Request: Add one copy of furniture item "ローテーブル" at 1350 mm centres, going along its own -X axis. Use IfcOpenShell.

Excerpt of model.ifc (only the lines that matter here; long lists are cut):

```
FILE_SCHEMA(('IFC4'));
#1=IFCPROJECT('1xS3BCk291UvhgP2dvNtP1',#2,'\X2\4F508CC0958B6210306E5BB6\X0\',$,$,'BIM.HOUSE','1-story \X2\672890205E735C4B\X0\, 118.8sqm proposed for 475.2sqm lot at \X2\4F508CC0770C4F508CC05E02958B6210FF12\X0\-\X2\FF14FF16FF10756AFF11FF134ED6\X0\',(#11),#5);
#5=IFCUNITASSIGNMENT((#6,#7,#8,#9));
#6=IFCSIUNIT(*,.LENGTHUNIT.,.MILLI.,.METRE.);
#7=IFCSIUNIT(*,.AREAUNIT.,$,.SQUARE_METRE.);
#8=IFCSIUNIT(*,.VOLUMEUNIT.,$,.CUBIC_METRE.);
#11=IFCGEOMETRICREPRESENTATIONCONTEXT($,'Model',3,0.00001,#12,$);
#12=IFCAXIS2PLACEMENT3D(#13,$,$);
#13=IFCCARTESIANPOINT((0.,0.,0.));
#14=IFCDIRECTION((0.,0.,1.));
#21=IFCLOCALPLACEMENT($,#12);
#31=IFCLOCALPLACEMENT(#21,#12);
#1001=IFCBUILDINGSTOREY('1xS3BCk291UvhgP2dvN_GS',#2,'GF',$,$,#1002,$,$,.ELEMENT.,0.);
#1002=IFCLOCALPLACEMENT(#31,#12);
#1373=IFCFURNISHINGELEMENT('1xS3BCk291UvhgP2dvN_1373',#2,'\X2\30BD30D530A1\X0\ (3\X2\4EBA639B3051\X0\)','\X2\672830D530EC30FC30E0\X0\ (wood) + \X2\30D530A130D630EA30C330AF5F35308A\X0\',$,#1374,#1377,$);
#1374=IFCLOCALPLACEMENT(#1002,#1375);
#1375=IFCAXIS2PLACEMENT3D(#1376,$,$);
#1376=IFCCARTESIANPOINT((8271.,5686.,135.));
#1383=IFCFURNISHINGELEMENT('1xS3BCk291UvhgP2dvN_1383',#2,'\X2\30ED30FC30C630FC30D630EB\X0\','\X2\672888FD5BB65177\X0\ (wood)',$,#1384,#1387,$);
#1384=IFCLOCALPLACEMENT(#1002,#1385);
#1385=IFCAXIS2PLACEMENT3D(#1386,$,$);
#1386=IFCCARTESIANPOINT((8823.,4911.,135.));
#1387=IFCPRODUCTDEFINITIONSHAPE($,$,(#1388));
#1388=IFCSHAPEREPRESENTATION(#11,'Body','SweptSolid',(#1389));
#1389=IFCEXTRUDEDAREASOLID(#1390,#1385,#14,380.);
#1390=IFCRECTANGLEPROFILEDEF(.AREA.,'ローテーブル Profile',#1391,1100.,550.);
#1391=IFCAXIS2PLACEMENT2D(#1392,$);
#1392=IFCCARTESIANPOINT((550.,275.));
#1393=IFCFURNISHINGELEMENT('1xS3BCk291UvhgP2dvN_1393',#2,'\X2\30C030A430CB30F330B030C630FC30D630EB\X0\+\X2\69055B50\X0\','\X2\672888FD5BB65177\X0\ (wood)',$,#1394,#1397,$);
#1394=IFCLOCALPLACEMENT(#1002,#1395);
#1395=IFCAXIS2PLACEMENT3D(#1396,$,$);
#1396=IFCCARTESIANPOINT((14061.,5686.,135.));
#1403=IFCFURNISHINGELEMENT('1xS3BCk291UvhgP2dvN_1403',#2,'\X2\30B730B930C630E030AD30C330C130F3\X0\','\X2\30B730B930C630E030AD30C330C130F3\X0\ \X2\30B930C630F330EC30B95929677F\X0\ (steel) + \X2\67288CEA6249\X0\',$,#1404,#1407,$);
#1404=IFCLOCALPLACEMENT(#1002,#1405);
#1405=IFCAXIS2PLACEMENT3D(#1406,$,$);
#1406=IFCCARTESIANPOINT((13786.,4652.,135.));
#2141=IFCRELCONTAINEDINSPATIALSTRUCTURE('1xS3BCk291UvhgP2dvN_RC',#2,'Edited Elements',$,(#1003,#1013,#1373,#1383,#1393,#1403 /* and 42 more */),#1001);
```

```python
import ifcopenshell
import ifcopenshell.api.geometry
import ifcopenshell.api.root
import ifcopenshell.util.element
import ifcopenshell.util.placement
import ifcopenshell.util.unit

model = ifcopenshell.open("model.ifc")
unit_scale = ifcopenshell.util.unit.calculate_unit_scale(model)


def reuse_history(source, copy):
    """copy_class also copies each property set's owner history, people and application; keep the originals."""
    for rel in copy.IsDefinedBy:
        if rel.is_a("IfcRelDefinesByProperties") and (history := rel.RelatingPropertyDefinition.OwnerHistory):
            rel.RelatingPropertyDefinition.OwnerHistory = source.OwnerHistory
            ifcopenshell.util.element.remove_deep2(model, history)


source = model.by_guid("1xS3BCk291UvhgP2dvN_1383")
base = ifcopenshell.util.placement.get_local_placement(source.ObjectPlacement)
step = -base[:3, 0] * 1.35 / unit_scale

for i in range(1, 2):
    copy = ifcopenshell.api.root.copy_class(model, product=source)
    copy.Representation = ifcopenshell.util.element.copy_deep(
        model, source.Representation, exclude=["IfcGeometricRepresentationContext", "IfcRepresentationMap"]
    )
    reuse_history(source, copy)
    matrix = base.copy()
    matrix[:3, 3] += i * step
    print("added at", matrix[:3, 3].round(3) + 0.0)
    ifcopenshell.api.geometry.edit_object_placement(model, product=copy, matrix=matrix, is_si=False)

model.write("model_rev.ifc")
```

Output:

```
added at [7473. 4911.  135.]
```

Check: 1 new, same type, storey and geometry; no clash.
